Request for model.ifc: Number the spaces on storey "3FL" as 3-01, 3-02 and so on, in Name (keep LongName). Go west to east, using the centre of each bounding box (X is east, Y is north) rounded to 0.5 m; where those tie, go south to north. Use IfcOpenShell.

First a look at what the model holds.

```python
import ifcopenshell
import ifcopenshell.util.element
import ifcopenshell.util.placement

model = ifcopenshell.open("model.ifc")
print(model.schema)
storey = next(s for s in model.by_type("IfcBuildingStorey") if s.Name == "3FL")
spaces = [e for e in ifcopenshell.util.element.get_decomposition(storey) if e.is_a("IfcSpace")]
for e in sorted(spaces, key=lambda e: e.id()):
    origin = ifcopenshell.util.placement.get_local_placement(e.ObjectPlacement)[:3, 3]
    print(e.id(), e.Name, e.LongName, origin.round(2) + 0.0, sep=" | ")
```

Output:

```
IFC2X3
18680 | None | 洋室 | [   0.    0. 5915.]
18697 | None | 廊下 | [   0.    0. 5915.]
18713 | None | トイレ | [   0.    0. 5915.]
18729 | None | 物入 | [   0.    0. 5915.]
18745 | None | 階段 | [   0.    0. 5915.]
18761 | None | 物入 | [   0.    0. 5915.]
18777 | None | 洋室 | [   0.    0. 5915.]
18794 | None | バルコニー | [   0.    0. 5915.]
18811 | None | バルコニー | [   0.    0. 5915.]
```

```python
import ifcopenshell
import ifcopenshell.geom
import ifcopenshell.util.element
import ifcopenshell.util.shape

model = ifcopenshell.open("model.ifc")
settings = ifcopenshell.geom.settings()
settings.set("use-world-coords", True)


def centre(element):
    shape = ifcopenshell.geom.create_shape(settings, element)
    return ifcopenshell.util.shape.get_bbox_centroid(shape.geometry)


storey = next(s for s in model.by_type("IfcBuildingStorey") if s.Name == "3FL")
spaces = [e for e in ifcopenshell.util.element.get_decomposition(storey) if e.is_a("IfcSpace")]

# Insertion points can sit at a corner or the storey origin, so sort by the geometry (in metres).
centres = {e: centre(e) for e in spaces}
spaces.sort(key=lambda e: (round(centres[e][0] / 0.5), centres[e][1]))

for i, e in enumerate(spaces, start=1):
    number = f"3-{i:02d}"
    e.Name = number
    print(e.id(), number)

model.write("model-out.ifc")
```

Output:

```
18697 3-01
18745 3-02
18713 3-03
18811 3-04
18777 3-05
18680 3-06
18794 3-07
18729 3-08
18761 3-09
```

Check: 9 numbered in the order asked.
